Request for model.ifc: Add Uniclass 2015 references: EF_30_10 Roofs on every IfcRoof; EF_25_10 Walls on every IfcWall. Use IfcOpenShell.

First a look at what the model holds.

```python
import ifcopenshell

model = ifcopenshell.open("model.ifc")
print(model.schema)
print("classifications:", [c.Name for c in model.by_type("IfcClassification")])
for ifc_class in ("IfcDoor", "IfcRoof", "IfcStair", "IfcWall", "IfcWindow"):
    print(ifc_class, len(model.by_type(ifc_class)))
```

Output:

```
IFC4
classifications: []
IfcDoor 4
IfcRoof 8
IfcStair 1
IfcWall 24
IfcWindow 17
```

```python
import ifcopenshell
import ifcopenshell.api.classification

model = ifcopenshell.open("model.ifc")

system = ifcopenshell.api.classification.add_classification(model, classification="Uniclass 2015")

codes = {
    "IfcRoof": ("EF_30_10", "Roofs"),
    "IfcWall": ("EF_25_10", "Walls"),
}
for ifc_class, (code, name) in codes.items():
    products = model.by_type(ifc_class)
    ifcopenshell.api.classification.add_reference(
        model, products=products, classification=system, identification=code, name=name
    )
    print(code, len(products))

model.write("model-out.ifc")
```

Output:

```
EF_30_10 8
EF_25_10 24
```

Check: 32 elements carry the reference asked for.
